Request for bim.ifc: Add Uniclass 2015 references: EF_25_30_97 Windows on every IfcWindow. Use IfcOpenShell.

First a look at what the model holds.

```python
import ifcopenshell

model = ifcopenshell.open("bim.ifc")
print(model.schema)
print("classifications:", [c.Name for c in model.by_type("IfcClassification")])
for ifc_class in ("IfcDoor", "IfcRoof", "IfcStair", "IfcWall", "IfcWindow"):
    print(ifc_class, len(model.by_type(ifc_class)))
```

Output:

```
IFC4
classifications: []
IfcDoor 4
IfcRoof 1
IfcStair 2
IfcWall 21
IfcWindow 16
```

```python
import ifcopenshell
import ifcopenshell.api.classification

model = ifcopenshell.open("bim.ifc")

system = ifcopenshell.api.classification.add_classification(model, classification="Uniclass 2015")

codes = {
    "IfcWindow": ("EF_25_30_97", "Windows"),
}
for ifc_class, (code, name) in codes.items():
    products = model.by_type(ifc_class)
    ifcopenshell.api.classification.add_reference(
        model, products=products, classification=system, identification=code, name=name
    )
    print(code, len(products))

model.write("bim-out.ifc")
```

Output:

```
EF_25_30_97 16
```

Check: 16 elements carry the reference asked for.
